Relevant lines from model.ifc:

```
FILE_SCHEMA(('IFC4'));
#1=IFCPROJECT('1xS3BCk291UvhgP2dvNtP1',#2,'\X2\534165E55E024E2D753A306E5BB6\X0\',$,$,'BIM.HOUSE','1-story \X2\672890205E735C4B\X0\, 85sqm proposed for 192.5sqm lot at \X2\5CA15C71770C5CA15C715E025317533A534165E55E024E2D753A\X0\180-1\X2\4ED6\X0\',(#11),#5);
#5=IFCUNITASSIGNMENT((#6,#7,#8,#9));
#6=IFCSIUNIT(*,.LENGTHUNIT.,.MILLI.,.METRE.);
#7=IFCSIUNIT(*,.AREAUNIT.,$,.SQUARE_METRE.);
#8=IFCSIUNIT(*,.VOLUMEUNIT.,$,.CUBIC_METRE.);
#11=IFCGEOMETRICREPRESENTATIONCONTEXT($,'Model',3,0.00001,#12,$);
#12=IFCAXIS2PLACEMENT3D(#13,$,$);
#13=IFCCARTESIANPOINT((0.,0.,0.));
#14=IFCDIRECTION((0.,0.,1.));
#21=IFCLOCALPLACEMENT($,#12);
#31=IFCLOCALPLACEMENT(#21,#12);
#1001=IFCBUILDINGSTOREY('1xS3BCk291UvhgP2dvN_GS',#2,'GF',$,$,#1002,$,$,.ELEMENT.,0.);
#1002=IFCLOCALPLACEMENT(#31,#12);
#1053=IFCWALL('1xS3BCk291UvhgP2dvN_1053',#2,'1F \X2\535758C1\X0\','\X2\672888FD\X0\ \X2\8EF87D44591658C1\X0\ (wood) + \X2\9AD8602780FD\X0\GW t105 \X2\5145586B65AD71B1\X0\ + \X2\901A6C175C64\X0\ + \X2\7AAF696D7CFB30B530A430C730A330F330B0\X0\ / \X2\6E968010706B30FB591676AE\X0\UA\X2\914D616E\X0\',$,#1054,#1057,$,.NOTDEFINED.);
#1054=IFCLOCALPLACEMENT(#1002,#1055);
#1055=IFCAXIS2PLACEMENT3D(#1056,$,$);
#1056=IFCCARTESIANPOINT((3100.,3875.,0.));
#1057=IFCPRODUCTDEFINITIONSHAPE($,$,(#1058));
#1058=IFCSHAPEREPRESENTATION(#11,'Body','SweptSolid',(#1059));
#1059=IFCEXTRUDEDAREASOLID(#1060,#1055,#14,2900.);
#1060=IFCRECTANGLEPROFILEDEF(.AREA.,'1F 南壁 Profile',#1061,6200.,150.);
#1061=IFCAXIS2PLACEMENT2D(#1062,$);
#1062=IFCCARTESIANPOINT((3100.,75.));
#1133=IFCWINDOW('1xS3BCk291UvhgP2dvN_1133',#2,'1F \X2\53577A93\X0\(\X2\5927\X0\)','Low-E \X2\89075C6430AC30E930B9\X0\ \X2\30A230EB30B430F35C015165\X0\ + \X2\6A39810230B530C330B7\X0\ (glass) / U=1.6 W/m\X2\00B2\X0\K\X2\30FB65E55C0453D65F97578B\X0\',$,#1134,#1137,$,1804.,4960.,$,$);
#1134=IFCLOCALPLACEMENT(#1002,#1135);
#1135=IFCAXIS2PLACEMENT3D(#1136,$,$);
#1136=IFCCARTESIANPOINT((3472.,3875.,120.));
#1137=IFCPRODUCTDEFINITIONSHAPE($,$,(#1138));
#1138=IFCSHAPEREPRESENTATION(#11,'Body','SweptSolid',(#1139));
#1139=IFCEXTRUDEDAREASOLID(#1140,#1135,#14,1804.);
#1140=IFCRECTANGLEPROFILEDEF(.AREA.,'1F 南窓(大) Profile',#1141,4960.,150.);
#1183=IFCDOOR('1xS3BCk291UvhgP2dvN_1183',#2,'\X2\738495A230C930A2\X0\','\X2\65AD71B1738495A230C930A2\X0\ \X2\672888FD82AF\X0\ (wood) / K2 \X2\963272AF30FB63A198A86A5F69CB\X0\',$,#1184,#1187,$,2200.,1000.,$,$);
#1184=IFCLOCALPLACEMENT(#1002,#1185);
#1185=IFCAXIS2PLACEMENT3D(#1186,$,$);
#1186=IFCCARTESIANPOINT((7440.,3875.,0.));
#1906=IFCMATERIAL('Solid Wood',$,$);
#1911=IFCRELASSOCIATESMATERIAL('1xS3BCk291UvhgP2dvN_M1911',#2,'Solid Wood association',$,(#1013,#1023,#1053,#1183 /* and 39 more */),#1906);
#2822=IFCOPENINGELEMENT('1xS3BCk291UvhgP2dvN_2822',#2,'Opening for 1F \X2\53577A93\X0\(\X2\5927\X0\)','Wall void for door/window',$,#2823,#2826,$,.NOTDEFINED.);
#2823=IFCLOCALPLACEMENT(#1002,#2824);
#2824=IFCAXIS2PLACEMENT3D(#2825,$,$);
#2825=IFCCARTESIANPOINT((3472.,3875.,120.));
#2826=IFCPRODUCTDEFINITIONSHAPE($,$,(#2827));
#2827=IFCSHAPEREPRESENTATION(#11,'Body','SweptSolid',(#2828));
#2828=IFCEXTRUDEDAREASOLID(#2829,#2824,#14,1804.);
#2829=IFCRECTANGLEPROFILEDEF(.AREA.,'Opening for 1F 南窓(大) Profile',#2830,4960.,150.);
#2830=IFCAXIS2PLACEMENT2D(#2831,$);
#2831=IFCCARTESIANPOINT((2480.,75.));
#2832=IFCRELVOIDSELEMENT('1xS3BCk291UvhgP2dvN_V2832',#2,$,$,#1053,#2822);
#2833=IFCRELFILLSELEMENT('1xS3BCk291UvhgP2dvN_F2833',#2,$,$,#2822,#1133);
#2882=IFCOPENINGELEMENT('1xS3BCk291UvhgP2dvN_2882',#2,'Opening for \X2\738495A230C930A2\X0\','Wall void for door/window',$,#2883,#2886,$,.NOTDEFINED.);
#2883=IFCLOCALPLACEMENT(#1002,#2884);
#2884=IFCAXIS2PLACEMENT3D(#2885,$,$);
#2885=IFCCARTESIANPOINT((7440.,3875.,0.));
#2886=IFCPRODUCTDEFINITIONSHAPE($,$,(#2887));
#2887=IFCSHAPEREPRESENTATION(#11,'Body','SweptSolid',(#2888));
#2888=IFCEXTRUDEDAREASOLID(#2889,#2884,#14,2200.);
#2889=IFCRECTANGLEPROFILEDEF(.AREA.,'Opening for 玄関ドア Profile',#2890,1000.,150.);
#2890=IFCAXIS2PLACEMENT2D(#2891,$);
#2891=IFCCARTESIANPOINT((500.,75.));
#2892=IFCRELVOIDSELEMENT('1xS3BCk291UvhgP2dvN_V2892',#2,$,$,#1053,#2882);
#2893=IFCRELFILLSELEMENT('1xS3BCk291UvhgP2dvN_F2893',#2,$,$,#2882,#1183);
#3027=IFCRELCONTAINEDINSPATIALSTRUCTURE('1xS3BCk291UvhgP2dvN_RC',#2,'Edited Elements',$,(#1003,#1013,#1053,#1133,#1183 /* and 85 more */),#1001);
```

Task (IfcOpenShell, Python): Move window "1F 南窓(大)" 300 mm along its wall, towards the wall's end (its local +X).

```python
import ifcopenshell
import ifcopenshell.api.geometry
import ifcopenshell.util.placement
import ifcopenshell.util.unit

model = ifcopenshell.open("model.ifc")
unit_scale = ifcopenshell.util.unit.calculate_unit_scale(model)

window = model.by_id(1133)
opening = window.FillsVoids[0].RelatingOpeningElement
wall = opening.VoidsElements[0].RelatingBuildingElement

wall_matrix = ifcopenshell.util.placement.get_local_placement(wall.ObjectPlacement)
shift = wall_matrix[:3, 0] * 0.3 / unit_scale
before = ifcopenshell.util.placement.get_local_placement(window.ObjectPlacement)[:3, 3].copy()

# The window is not placed relative to its opening, so move both.
for product in (opening, window):
    matrix = ifcopenshell.util.placement.get_local_placement(product.ObjectPlacement)
    matrix[:3, 3] += shift
    ifcopenshell.api.geometry.edit_object_placement(model, product=product, matrix=matrix, is_si=False)

after = ifcopenshell.util.placement.get_local_placement(window.ObjectPlacement)[:3, 3]
print("window moved by", (after - before).round(3) + 0.0)

model.write("model_updated.ifc")
```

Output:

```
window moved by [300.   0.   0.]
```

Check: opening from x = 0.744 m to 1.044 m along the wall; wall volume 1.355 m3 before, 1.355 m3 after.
